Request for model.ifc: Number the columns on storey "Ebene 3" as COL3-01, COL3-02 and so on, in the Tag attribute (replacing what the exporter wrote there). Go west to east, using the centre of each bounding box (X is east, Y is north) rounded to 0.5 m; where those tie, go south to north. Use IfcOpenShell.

First a look at what the model holds.

```python
import ifcopenshell
import ifcopenshell.util.element
import ifcopenshell.util.placement

model = ifcopenshell.open("model.ifc")
print(model.schema)
storey = next(s for s in model.by_type("IfcBuildingStorey") if s.Name == "Ebene 3")
columns = [e for e in ifcopenshell.util.element.get_decomposition(storey) if e.is_a("IfcColumn")]
for e in sorted(columns, key=lambda e: e.id()):
    origin = ifcopenshell.util.placement.get_local_placement(e.ObjectPlacement)[:3, 3]
    print(e.id(), e.Tag, e.Name, origin.round(2) + 0.0, sep=" | ")
```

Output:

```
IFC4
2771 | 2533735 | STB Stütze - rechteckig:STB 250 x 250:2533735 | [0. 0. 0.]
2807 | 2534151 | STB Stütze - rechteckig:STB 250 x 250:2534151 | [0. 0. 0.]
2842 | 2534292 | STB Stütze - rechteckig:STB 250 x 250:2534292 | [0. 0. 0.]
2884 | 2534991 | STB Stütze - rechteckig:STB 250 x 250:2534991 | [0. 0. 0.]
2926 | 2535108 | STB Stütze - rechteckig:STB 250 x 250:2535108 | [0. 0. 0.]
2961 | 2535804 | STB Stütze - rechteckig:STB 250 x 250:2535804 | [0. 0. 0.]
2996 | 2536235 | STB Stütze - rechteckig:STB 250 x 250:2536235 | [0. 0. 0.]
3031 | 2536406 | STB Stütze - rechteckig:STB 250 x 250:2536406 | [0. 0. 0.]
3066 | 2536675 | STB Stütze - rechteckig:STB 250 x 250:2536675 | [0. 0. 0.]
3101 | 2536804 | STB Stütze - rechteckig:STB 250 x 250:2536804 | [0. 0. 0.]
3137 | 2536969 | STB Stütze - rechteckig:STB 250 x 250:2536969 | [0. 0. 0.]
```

```python
import ifcopenshell
import ifcopenshell.geom
import ifcopenshell.util.element
import ifcopenshell.util.shape

model = ifcopenshell.open("model.ifc")
settings = ifcopenshell.geom.settings()
settings.set("use-world-coords", True)


def centre(element):
    shape = ifcopenshell.geom.create_shape(settings, element)
    return ifcopenshell.util.shape.get_bbox_centroid(shape.geometry)


storey = next(s for s in model.by_type("IfcBuildingStorey") if s.Name == "Ebene 3")
columns = [e for e in ifcopenshell.util.element.get_decomposition(storey) if e.is_a("IfcColumn")]

# Insertion points can sit at a corner or the storey origin, so sort by the geometry (in metres).
centres = {e: centre(e) for e in columns}
columns.sort(key=lambda e: (round(centres[e][0] / 0.5), centres[e][1]))

for i, e in enumerate(columns, start=1):
    number = f"COL3-{i:02d}"
    e.Tag = number
    print(e.id(), number)

model.write("model_v2.ifc")
```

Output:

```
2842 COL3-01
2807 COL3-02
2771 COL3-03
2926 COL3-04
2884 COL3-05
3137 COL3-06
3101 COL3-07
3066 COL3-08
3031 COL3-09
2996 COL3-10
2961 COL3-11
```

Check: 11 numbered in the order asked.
